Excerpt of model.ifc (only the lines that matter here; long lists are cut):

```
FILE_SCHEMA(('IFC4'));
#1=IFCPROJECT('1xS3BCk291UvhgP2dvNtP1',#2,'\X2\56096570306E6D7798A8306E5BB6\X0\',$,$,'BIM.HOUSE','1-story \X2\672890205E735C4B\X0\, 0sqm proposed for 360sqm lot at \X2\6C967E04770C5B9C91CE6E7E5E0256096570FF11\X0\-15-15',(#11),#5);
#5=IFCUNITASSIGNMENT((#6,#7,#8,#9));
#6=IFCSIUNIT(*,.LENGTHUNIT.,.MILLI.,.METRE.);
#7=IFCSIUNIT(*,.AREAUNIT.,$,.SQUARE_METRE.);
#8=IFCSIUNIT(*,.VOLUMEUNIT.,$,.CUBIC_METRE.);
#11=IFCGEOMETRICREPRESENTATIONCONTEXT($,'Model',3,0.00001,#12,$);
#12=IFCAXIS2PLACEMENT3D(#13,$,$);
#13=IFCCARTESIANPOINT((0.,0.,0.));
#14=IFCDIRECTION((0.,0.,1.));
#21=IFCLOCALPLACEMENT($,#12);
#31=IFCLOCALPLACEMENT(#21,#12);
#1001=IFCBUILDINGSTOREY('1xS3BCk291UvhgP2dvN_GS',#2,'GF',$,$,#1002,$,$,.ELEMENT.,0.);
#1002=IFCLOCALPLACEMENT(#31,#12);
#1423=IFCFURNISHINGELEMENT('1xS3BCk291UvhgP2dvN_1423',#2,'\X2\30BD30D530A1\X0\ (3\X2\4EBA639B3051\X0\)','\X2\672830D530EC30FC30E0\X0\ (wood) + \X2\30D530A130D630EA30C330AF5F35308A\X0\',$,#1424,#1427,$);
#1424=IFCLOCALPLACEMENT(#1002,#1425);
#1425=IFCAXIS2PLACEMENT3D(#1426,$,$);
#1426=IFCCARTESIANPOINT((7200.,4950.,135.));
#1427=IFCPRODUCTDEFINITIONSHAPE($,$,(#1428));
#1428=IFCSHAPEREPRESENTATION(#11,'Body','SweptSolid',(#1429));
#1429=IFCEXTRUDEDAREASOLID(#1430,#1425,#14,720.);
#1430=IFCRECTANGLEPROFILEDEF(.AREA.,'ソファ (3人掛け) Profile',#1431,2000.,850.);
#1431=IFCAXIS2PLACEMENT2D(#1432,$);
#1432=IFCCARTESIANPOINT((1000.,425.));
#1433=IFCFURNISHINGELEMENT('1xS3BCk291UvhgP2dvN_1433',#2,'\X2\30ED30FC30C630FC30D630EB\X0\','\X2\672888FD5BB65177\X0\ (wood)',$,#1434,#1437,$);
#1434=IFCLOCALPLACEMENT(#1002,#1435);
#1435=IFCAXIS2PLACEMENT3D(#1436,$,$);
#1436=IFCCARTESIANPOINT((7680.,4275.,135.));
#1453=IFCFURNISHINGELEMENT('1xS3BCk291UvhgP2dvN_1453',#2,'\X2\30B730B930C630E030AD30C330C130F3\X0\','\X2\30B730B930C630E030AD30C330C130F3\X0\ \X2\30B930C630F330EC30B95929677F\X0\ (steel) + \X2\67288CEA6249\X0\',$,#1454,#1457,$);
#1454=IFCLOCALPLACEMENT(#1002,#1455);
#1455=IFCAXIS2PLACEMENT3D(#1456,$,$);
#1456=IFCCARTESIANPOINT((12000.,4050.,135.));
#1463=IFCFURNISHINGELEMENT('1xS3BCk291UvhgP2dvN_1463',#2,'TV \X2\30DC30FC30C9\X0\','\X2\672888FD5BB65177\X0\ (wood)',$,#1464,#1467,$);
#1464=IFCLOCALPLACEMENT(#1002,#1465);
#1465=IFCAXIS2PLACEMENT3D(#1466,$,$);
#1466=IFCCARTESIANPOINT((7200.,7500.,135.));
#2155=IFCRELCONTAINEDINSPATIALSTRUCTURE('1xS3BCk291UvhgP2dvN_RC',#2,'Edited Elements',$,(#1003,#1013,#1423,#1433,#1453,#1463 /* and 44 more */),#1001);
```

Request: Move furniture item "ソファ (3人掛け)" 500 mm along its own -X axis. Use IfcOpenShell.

```python
import ifcopenshell
import ifcopenshell.api.geometry
import ifcopenshell.util.placement

model = ifcopenshell.open("model.ifc")

item = model.by_guid("1xS3BCk291UvhgP2dvN_1423")
matrix = ifcopenshell.util.placement.get_local_placement(item.ObjectPlacement)
matrix[:3, 3] -= matrix[:3, 0] * 500.0
ifcopenshell.api.geometry.edit_object_placement(model, product=item, matrix=matrix, is_si=False)

print(ifcopenshell.util.placement.get_local_placement(item.ObjectPlacement).round(3) + 0.0)

model.write("model_updated.ifc")
```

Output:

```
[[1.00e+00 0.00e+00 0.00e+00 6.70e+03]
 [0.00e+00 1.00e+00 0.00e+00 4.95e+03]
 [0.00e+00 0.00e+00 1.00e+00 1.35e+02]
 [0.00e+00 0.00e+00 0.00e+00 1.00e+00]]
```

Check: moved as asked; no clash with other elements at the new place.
